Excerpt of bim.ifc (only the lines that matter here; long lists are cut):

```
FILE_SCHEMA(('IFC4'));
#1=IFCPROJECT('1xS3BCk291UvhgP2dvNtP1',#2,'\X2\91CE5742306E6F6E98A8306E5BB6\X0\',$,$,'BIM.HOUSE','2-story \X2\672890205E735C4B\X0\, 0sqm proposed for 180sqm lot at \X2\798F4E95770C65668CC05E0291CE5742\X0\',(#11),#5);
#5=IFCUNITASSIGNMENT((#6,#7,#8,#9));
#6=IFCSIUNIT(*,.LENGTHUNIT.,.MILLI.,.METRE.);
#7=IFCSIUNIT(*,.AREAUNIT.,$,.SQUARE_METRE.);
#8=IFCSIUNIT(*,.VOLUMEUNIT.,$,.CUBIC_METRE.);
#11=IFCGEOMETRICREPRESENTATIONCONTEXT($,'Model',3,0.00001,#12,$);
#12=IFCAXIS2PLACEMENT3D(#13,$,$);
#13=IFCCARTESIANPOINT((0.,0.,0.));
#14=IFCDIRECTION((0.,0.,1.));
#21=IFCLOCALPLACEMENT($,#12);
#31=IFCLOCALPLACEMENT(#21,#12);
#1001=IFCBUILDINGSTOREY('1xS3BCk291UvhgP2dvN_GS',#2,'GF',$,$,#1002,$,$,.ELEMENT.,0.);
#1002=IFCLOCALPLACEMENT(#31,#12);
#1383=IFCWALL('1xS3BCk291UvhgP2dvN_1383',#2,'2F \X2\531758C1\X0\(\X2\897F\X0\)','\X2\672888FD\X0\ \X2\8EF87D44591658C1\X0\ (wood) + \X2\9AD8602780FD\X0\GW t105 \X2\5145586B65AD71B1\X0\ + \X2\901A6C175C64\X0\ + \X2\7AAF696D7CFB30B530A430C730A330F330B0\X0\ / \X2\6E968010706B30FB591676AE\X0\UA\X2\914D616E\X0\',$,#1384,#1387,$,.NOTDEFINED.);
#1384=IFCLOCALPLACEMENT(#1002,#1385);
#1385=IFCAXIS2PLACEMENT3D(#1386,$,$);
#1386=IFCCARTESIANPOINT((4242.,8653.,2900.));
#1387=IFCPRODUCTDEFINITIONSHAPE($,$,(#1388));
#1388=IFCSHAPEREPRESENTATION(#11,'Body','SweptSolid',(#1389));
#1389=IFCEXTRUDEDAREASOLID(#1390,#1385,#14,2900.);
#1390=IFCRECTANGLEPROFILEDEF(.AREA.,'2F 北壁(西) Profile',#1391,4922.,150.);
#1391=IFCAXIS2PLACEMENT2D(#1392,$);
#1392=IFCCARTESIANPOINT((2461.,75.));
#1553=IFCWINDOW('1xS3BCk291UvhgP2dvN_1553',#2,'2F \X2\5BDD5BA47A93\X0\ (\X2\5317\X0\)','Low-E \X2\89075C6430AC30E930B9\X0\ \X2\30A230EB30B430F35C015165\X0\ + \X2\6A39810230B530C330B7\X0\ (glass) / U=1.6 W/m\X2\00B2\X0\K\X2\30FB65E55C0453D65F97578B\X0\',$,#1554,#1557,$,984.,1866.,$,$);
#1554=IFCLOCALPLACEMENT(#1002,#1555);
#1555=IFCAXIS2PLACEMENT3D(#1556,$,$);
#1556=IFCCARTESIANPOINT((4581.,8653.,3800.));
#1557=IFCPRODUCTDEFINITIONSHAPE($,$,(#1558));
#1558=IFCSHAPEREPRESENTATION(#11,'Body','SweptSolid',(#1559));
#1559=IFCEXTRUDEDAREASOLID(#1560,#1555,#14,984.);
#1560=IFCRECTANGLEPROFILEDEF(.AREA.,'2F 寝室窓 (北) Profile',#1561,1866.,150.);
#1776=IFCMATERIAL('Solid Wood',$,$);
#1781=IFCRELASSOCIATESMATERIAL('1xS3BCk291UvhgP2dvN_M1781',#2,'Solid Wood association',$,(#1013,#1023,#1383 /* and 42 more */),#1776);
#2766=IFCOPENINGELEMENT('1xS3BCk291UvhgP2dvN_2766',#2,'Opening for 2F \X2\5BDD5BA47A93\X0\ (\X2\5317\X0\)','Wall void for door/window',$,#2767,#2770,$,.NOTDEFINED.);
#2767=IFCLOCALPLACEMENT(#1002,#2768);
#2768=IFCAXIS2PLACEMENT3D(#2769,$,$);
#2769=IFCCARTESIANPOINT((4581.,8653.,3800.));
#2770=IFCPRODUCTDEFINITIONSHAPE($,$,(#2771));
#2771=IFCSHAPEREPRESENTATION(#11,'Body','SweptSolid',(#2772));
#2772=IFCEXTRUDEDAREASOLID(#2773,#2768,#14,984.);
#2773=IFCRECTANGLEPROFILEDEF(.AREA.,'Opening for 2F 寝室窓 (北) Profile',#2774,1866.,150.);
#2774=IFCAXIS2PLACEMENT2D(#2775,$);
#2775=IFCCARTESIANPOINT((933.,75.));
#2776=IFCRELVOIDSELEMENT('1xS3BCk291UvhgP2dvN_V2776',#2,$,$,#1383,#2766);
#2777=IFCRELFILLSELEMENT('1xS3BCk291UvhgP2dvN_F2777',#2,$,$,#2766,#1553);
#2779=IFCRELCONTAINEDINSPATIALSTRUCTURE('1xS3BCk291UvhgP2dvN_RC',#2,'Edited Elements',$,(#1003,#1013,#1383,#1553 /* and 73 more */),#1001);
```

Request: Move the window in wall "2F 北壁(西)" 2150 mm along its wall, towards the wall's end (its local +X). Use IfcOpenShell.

```python
import ifcopenshell
import ifcopenshell.api.geometry
import ifcopenshell.util.placement
import ifcopenshell.util.unit

model = ifcopenshell.open("bim.ifc")
unit_scale = ifcopenshell.util.unit.calculate_unit_scale(model)

window = model.by_guid("1xS3BCk291UvhgP2dvN_1553")
opening = window.FillsVoids[0].RelatingOpeningElement
wall = opening.VoidsElements[0].RelatingBuildingElement

wall_matrix = ifcopenshell.util.placement.get_local_placement(wall.ObjectPlacement)
shift = wall_matrix[:3, 0] * 2.15 / unit_scale
before = ifcopenshell.util.placement.get_local_placement(window.ObjectPlacement)[:3, 3].copy()

# The window is not placed relative to its opening, so move both.
for product in (opening, window):
    matrix = ifcopenshell.util.placement.get_local_placement(product.ObjectPlacement)
    matrix[:3, 3] += shift
    ifcopenshell.api.geometry.edit_object_placement(model, product=product, matrix=matrix, is_si=False)

after = ifcopenshell.util.placement.get_local_placement(window.ObjectPlacement)[:3, 3]
print("window moved by", (after - before).round(3) + 0.0)

model.write("bim-out.ifc")
```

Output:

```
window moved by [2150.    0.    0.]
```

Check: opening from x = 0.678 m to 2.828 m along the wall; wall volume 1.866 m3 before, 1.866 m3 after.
